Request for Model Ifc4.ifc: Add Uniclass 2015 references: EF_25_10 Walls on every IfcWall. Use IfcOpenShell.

First a look at what the model holds.

```python
import ifcopenshell

model = ifcopenshell.open("Model Ifc4.ifc")
print(model.schema)
print("classifications:", [c.Name for c in model.by_type("IfcClassification")])
for ifc_class in ("IfcDoor", "IfcRoof", "IfcStair", "IfcWall", "IfcWindow"):
    print(ifc_class, len(model.by_type(ifc_class)))
```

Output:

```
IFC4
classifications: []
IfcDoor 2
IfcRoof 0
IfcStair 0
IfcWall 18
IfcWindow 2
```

```python
import ifcopenshell
import ifcopenshell.api.classification

model = ifcopenshell.open("Model Ifc4.ifc")

system = ifcopenshell.api.classification.add_classification(model, classification="Uniclass 2015")

codes = {
    "IfcWall": ("EF_25_10", "Walls"),
}
for ifc_class, (code, name) in codes.items():
    products = model.by_type(ifc_class)
    ifcopenshell.api.classification.add_reference(
        model, products=products, classification=system, identification=code, name=name
    )
    print(code, len(products))

model.write("Model Ifc4-out.ifc")
```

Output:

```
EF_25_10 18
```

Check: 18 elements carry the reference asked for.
